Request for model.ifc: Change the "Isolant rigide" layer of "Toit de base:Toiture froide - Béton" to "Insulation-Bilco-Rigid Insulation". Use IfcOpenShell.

First a look at what the model holds.

```python
import ifcopenshell
import ifcopenshell.util.element

model = ifcopenshell.open("model.ifc")
print(model.schema)
for layer_set in model.by_type("IfcMaterialLayerSet"):
    if layer_set.LayerSetName == "Toit de base:Toiture froide - Béton":
        for layer in layer_set.MaterialLayers:
            print(layer.id(), layer.Material and layer.Material.Name, layer.LayerThickness, sep=" | ")
        print(len(ifcopenshell.util.element.get_elements_by_material(model, layer_set)), "elements and types use it")
print(sorted(m.Name for m in model.by_type("IfcMaterial") if m.Name)[:60])
```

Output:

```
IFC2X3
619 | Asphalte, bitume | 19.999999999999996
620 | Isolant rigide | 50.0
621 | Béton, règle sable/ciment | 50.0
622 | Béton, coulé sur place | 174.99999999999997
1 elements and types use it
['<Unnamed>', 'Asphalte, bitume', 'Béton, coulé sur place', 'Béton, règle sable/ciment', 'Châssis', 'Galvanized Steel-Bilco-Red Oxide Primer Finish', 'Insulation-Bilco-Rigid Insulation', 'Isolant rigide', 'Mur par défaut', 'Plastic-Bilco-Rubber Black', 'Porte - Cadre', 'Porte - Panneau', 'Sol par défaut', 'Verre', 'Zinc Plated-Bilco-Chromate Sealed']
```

```python
import ifcopenshell
import ifcopenshell.api.material

model = ifcopenshell.open("model.ifc")

layer_set = next(s for s in model.by_type("IfcMaterialLayerSet") if s.LayerSetName == "Toit de base:Toiture froide - Béton")
layer = next(l for l in layer_set.MaterialLayers if l.Material and l.Material.Name == "Isolant rigide")
material = next(m for m in model.by_type("IfcMaterial") if m.Name == "Insulation-Bilco-Rigid Insulation")

# Point this one layer at the other material; renaming the old one would change it everywhere.
ifcopenshell.api.material.edit_layer(model, layer=layer, attributes={}, material=material)

print([l.Material.Name if l.Material else None for l in layer_set.MaterialLayers])

model.write("model_rev.ifc")
```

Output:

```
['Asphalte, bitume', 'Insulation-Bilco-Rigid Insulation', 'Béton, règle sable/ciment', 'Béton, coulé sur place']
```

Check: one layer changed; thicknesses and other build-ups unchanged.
